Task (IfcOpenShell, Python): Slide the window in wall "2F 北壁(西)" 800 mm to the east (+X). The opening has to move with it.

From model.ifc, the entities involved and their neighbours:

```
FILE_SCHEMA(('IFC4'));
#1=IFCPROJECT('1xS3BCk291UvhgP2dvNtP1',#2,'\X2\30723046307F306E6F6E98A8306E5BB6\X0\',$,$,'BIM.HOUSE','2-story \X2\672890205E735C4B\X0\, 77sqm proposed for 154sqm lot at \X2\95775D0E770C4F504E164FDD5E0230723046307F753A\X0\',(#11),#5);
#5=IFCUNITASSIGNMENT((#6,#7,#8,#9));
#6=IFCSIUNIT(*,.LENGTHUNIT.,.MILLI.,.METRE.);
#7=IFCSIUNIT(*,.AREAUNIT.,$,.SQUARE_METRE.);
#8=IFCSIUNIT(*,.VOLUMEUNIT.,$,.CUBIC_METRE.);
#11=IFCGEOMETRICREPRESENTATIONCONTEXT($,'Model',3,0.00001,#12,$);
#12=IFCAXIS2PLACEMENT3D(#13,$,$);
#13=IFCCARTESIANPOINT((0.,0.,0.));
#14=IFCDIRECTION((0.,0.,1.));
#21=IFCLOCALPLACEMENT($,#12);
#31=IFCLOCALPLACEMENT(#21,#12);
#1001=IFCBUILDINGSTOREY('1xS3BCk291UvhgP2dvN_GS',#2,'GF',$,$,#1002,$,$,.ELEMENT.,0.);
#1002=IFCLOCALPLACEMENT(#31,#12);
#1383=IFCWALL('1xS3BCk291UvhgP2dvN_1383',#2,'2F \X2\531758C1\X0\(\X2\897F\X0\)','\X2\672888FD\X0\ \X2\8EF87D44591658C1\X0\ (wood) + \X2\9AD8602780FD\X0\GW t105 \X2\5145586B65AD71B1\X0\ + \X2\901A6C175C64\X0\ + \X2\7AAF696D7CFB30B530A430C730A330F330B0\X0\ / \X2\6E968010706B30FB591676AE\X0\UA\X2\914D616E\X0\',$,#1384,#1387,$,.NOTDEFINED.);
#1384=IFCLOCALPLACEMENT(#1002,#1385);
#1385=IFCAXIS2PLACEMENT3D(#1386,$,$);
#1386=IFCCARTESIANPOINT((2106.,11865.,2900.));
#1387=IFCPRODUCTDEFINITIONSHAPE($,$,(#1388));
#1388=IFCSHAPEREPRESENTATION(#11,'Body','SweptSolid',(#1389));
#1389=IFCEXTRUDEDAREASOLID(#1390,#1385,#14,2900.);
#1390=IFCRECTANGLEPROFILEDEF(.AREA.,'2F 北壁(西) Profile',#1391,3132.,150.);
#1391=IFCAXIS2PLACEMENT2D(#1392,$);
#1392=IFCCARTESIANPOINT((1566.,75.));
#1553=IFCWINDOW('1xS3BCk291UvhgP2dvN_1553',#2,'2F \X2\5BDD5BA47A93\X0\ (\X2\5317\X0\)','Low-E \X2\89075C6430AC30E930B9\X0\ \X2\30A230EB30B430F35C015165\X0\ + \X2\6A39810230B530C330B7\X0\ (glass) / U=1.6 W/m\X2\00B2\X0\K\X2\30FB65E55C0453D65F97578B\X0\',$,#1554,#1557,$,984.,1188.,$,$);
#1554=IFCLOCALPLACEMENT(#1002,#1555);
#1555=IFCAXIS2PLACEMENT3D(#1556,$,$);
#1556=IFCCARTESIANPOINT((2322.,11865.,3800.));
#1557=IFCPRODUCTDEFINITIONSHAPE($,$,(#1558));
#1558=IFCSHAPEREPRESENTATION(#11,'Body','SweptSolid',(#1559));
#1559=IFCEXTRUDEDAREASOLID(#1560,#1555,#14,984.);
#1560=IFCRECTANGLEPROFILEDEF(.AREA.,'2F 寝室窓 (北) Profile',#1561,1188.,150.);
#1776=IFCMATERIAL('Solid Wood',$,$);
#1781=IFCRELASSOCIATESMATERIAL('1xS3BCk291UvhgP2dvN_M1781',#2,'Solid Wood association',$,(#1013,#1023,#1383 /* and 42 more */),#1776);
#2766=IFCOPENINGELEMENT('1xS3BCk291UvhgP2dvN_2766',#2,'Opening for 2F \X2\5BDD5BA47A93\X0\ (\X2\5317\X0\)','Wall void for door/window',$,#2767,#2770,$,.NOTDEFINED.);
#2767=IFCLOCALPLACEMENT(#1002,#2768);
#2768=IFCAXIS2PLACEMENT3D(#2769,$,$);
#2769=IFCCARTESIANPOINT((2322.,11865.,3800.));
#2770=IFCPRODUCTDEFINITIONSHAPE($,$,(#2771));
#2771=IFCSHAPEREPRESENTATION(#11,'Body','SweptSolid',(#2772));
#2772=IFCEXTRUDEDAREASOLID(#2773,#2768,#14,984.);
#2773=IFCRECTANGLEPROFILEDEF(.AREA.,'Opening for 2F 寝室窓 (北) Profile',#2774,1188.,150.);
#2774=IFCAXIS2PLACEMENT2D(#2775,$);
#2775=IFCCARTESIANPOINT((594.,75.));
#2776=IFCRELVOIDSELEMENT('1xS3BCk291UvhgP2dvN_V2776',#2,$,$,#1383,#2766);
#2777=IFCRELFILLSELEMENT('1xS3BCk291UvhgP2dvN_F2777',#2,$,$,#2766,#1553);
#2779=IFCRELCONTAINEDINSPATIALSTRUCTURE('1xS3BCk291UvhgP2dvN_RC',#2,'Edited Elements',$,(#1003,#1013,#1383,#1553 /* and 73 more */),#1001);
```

```python
import ifcopenshell
import ifcopenshell.api.geometry
import ifcopenshell.util.placement
import ifcopenshell.util.unit

model = ifcopenshell.open("model.ifc")
unit_scale = ifcopenshell.util.unit.calculate_unit_scale(model)

window = model.by_guid("1xS3BCk291UvhgP2dvN_1553")
opening = window.FillsVoids[0].RelatingOpeningElement
wall = opening.VoidsElements[0].RelatingBuildingElement

wall_matrix = ifcopenshell.util.placement.get_local_placement(wall.ObjectPlacement)
shift = wall_matrix[:3, 0] * 0.8 / unit_scale
before = ifcopenshell.util.placement.get_local_placement(window.ObjectPlacement)[:3, 3].copy()

# The window is not placed relative to its opening, so move both.
for product in (opening, window):
    matrix = ifcopenshell.util.placement.get_local_placement(product.ObjectPlacement)
    matrix[:3, 3] += shift
    ifcopenshell.api.geometry.edit_object_placement(model, product=product, matrix=matrix, is_si=False)

after = ifcopenshell.util.placement.get_local_placement(window.ObjectPlacement)[:3, 3]
print("window moved by", (after - before).round(3) + 0.0)

model.write("model_updated.ifc")
```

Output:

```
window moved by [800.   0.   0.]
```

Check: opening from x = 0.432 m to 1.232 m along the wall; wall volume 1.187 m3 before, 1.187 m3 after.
